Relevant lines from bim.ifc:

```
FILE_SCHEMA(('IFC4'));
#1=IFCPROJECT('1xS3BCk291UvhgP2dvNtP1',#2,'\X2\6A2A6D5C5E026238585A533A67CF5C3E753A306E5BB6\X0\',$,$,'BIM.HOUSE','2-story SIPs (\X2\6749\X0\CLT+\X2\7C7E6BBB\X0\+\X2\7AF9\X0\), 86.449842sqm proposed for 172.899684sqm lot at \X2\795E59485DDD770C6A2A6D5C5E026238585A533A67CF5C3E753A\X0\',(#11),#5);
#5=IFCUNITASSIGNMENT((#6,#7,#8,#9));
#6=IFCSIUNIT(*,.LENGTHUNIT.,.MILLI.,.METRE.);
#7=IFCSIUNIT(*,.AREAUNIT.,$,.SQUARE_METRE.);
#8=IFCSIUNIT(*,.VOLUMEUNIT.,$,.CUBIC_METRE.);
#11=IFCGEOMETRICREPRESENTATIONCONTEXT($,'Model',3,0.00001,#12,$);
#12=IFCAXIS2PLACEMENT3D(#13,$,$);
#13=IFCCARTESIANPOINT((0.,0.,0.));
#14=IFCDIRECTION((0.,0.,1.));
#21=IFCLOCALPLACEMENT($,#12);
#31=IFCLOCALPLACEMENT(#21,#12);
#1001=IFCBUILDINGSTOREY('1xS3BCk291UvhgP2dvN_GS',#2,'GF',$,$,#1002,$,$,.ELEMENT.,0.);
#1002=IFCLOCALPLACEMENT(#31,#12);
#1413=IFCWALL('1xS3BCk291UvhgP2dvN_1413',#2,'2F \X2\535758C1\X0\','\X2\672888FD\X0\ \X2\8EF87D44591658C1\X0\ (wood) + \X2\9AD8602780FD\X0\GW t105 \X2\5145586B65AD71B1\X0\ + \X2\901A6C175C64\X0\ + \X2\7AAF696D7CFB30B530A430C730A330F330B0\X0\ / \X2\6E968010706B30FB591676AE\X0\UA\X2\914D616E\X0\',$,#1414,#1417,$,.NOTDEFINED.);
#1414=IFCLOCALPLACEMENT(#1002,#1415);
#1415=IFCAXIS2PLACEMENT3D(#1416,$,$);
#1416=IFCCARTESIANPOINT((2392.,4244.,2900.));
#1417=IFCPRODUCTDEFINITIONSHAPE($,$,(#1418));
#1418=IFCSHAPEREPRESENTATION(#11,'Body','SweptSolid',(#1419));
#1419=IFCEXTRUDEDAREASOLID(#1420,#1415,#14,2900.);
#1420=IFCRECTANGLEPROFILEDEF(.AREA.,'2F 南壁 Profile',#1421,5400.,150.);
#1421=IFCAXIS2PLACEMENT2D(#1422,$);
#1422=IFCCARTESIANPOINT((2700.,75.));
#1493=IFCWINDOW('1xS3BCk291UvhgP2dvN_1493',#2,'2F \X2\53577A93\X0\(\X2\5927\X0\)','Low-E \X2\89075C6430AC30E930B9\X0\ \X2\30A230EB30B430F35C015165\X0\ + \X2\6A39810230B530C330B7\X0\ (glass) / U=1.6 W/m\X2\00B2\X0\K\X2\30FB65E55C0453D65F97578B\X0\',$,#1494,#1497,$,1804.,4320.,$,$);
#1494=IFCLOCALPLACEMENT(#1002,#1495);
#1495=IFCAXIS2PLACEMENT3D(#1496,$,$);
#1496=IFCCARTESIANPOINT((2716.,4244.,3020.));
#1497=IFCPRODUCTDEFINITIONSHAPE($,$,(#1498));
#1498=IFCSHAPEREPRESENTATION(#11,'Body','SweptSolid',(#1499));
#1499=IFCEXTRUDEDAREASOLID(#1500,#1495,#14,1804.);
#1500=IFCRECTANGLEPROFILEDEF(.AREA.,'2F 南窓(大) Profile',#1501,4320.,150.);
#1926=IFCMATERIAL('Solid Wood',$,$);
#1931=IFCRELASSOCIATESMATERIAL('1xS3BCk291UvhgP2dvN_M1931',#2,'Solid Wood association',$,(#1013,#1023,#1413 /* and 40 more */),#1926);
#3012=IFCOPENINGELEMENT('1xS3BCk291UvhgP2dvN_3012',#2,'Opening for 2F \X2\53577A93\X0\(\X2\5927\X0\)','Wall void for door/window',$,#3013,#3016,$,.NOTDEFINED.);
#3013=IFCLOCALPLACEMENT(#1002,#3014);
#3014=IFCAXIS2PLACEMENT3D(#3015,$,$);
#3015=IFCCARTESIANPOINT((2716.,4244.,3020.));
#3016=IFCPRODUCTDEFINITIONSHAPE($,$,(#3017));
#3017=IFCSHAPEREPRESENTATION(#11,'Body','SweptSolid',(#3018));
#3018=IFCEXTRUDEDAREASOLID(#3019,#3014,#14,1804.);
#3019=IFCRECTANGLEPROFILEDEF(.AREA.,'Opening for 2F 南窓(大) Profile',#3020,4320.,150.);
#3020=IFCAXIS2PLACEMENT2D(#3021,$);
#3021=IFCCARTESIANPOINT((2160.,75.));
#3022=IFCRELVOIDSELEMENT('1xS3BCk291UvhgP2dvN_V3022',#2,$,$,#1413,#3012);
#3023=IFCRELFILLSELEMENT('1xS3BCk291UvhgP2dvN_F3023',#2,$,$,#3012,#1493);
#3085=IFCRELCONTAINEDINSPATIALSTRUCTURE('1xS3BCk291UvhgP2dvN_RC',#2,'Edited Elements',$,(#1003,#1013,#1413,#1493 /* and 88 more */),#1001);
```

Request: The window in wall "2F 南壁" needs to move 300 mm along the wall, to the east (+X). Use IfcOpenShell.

```python
import ifcopenshell
import ifcopenshell.api.geometry
import ifcopenshell.util.placement

model = ifcopenshell.open("bim.ifc")

window = model.by_id(1493)
opening = window.FillsVoids[0].RelatingOpeningElement
wall = opening.VoidsElements[0].RelatingBuildingElement

wall_matrix = ifcopenshell.util.placement.get_local_placement(wall.ObjectPlacement)
shift = wall_matrix[:3, 0] * 300.0
before = ifcopenshell.util.placement.get_local_placement(window.ObjectPlacement)[:3, 3].copy()

# The window is not placed relative to its opening, so move both.
for product in (opening, window):
    matrix = ifcopenshell.util.placement.get_local_placement(product.ObjectPlacement)
    matrix[:3, 3] += shift
    ifcopenshell.api.geometry.edit_object_placement(model, product=product, matrix=matrix, is_si=False)

after = ifcopenshell.util.placement.get_local_placement(window.ObjectPlacement)[:3, 3]
print("window moved by", (after - before).round(3) + 0.0)

model.write("bim_v2.ifc")
```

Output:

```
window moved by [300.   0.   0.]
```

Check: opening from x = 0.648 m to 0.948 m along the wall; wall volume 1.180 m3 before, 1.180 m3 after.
